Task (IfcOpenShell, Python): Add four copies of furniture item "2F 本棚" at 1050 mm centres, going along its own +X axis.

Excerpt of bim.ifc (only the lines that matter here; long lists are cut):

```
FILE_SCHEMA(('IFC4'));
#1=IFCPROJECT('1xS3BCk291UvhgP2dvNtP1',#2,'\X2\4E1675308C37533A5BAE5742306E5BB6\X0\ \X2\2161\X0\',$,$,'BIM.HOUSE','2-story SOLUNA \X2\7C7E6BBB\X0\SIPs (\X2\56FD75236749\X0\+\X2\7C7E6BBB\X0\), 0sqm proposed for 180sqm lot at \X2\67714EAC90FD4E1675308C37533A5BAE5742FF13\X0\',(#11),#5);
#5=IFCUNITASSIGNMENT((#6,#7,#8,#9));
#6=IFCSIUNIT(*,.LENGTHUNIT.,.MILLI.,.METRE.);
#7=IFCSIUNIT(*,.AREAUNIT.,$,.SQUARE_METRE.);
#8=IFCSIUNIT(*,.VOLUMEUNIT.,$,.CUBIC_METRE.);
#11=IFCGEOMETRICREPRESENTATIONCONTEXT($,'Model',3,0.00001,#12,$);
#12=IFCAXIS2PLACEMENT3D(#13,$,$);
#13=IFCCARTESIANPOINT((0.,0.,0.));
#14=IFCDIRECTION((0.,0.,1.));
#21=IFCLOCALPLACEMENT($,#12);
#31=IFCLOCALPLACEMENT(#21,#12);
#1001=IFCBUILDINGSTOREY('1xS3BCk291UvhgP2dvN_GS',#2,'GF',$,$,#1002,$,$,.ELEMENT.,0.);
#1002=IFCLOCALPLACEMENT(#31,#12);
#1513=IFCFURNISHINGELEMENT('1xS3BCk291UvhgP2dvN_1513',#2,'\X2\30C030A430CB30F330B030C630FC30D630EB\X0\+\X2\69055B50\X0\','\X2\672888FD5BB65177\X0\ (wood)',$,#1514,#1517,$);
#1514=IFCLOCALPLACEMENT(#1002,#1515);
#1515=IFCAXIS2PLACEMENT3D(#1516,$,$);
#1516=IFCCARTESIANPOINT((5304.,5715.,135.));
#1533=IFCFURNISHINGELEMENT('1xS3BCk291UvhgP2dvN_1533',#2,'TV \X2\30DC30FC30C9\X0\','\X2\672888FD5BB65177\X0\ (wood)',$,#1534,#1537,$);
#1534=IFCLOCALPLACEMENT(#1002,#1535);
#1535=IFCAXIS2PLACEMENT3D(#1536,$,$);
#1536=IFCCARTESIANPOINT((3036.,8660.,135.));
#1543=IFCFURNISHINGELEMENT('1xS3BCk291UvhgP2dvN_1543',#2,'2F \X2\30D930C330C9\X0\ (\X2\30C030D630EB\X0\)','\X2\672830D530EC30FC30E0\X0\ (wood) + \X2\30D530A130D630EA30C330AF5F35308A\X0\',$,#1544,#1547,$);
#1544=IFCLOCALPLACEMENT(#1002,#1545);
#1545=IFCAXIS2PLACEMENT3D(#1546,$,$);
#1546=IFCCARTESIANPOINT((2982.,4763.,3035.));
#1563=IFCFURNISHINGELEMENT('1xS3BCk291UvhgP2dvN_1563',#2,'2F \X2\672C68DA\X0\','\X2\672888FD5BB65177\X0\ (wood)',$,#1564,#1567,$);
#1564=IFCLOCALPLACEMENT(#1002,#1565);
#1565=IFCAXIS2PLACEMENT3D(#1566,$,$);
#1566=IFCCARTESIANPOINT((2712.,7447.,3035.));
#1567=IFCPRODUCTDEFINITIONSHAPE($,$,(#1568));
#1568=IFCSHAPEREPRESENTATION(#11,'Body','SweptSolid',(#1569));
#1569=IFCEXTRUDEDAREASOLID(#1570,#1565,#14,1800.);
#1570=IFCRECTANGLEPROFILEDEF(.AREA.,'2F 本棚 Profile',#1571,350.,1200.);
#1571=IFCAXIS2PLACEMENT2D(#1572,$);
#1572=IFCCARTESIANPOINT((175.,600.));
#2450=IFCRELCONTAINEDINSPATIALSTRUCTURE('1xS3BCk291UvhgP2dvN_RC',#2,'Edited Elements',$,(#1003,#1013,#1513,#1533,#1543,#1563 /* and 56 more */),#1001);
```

```python
import ifcopenshell
import ifcopenshell.api.geometry
import ifcopenshell.api.root
import ifcopenshell.util.element
import ifcopenshell.util.placement

model = ifcopenshell.open("bim.ifc")


def reuse_history(source, copy):
    """copy_class also copies each property set's owner history, people and application; keep the originals."""
    for rel in copy.IsDefinedBy:
        if rel.is_a("IfcRelDefinesByProperties") and (history := rel.RelatingPropertyDefinition.OwnerHistory):
            rel.RelatingPropertyDefinition.OwnerHistory = source.OwnerHistory
            ifcopenshell.util.element.remove_deep2(model, history)


source = model.by_id(1563)
base = ifcopenshell.util.placement.get_local_placement(source.ObjectPlacement)
step = base[:3, 0] * 1050.0

for i in range(1, 5):
    copy = ifcopenshell.api.root.copy_class(model, product=source)
    copy.Representation = ifcopenshell.util.element.copy_deep(
        model, source.Representation, exclude=["IfcGeometricRepresentationContext", "IfcRepresentationMap"]
    )
    reuse_history(source, copy)
    matrix = base.copy()
    matrix[:3, 3] += i * step
    print("added at", matrix[:3, 3].round(3) + 0.0)
    ifcopenshell.api.geometry.edit_object_placement(model, product=copy, matrix=matrix, is_si=False)

model.write("bim_edited.ifc")
```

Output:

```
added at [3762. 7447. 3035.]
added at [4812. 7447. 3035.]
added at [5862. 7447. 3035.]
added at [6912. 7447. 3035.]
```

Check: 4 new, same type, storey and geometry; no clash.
